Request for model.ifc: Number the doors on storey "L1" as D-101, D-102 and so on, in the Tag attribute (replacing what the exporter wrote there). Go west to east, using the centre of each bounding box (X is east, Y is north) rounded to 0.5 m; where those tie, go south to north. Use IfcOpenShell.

First a look at what the model holds.

```python
import ifcopenshell
import ifcopenshell.util.element
import ifcopenshell.util.placement

model = ifcopenshell.open("model.ifc")
print(model.schema)
storey = next(s for s in model.by_type("IfcBuildingStorey") if s.Name == "L1")
doors = [e for e in ifcopenshell.util.element.get_decomposition(storey) if e.is_a("IfcDoor")]
for e in sorted(doors, key=lambda e: e.id()):
    origin = ifcopenshell.util.placement.get_local_placement(e.ObjectPlacement)[:3, 3]
    print(e.id(), e.Tag, e.Name, origin.round(2) + 0.0, sep=" | ")
```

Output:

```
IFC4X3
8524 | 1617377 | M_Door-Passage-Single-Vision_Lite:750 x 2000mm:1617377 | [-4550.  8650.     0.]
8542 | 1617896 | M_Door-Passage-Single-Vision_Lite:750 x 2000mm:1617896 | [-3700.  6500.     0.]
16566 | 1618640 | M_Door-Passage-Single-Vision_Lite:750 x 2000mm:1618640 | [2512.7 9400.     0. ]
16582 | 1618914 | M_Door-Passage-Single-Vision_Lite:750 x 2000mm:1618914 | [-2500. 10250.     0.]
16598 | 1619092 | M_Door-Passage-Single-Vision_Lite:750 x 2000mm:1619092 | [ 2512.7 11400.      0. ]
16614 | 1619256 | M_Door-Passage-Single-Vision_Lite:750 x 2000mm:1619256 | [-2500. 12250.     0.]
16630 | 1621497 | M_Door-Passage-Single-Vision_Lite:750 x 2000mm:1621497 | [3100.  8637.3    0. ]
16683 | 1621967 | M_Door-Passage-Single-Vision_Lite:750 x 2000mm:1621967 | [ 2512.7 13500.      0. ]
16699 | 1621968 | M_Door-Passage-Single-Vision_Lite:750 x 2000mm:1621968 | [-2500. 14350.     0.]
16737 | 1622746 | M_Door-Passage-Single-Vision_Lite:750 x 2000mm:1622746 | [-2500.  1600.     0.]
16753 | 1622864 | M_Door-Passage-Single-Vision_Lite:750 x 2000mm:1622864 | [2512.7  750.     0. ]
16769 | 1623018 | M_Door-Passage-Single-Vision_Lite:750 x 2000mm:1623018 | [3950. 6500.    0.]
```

```python
import ifcopenshell
import ifcopenshell.geom
import ifcopenshell.util.element
import ifcopenshell.util.shape

model = ifcopenshell.open("model.ifc")
settings = ifcopenshell.geom.settings()
settings.set("use-world-coords", True)


def centre(element):
    shape = ifcopenshell.geom.create_shape(settings, element)
    return ifcopenshell.util.shape.get_bbox_centroid(shape.geometry)


storey = next(s for s in model.by_type("IfcBuildingStorey") if s.Name == "L1")
doors = [e for e in ifcopenshell.util.element.get_decomposition(storey) if e.is_a("IfcDoor")]

# Insertion points can sit at a corner or the storey origin, so sort by the geometry (in metres).
centres = {e: centre(e) for e in doors}
doors.sort(key=lambda e: (round(centres[e][0] / 0.5), centres[e][1]))

for i, e in enumerate(doors, start=1):
    number = f"D-1{i:02d}"
    e.Tag = number
    print(e.id(), number)

model.write("model_updated.ifc")
```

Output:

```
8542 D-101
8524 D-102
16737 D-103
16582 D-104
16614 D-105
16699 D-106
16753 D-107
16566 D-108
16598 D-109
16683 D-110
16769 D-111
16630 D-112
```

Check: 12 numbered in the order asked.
